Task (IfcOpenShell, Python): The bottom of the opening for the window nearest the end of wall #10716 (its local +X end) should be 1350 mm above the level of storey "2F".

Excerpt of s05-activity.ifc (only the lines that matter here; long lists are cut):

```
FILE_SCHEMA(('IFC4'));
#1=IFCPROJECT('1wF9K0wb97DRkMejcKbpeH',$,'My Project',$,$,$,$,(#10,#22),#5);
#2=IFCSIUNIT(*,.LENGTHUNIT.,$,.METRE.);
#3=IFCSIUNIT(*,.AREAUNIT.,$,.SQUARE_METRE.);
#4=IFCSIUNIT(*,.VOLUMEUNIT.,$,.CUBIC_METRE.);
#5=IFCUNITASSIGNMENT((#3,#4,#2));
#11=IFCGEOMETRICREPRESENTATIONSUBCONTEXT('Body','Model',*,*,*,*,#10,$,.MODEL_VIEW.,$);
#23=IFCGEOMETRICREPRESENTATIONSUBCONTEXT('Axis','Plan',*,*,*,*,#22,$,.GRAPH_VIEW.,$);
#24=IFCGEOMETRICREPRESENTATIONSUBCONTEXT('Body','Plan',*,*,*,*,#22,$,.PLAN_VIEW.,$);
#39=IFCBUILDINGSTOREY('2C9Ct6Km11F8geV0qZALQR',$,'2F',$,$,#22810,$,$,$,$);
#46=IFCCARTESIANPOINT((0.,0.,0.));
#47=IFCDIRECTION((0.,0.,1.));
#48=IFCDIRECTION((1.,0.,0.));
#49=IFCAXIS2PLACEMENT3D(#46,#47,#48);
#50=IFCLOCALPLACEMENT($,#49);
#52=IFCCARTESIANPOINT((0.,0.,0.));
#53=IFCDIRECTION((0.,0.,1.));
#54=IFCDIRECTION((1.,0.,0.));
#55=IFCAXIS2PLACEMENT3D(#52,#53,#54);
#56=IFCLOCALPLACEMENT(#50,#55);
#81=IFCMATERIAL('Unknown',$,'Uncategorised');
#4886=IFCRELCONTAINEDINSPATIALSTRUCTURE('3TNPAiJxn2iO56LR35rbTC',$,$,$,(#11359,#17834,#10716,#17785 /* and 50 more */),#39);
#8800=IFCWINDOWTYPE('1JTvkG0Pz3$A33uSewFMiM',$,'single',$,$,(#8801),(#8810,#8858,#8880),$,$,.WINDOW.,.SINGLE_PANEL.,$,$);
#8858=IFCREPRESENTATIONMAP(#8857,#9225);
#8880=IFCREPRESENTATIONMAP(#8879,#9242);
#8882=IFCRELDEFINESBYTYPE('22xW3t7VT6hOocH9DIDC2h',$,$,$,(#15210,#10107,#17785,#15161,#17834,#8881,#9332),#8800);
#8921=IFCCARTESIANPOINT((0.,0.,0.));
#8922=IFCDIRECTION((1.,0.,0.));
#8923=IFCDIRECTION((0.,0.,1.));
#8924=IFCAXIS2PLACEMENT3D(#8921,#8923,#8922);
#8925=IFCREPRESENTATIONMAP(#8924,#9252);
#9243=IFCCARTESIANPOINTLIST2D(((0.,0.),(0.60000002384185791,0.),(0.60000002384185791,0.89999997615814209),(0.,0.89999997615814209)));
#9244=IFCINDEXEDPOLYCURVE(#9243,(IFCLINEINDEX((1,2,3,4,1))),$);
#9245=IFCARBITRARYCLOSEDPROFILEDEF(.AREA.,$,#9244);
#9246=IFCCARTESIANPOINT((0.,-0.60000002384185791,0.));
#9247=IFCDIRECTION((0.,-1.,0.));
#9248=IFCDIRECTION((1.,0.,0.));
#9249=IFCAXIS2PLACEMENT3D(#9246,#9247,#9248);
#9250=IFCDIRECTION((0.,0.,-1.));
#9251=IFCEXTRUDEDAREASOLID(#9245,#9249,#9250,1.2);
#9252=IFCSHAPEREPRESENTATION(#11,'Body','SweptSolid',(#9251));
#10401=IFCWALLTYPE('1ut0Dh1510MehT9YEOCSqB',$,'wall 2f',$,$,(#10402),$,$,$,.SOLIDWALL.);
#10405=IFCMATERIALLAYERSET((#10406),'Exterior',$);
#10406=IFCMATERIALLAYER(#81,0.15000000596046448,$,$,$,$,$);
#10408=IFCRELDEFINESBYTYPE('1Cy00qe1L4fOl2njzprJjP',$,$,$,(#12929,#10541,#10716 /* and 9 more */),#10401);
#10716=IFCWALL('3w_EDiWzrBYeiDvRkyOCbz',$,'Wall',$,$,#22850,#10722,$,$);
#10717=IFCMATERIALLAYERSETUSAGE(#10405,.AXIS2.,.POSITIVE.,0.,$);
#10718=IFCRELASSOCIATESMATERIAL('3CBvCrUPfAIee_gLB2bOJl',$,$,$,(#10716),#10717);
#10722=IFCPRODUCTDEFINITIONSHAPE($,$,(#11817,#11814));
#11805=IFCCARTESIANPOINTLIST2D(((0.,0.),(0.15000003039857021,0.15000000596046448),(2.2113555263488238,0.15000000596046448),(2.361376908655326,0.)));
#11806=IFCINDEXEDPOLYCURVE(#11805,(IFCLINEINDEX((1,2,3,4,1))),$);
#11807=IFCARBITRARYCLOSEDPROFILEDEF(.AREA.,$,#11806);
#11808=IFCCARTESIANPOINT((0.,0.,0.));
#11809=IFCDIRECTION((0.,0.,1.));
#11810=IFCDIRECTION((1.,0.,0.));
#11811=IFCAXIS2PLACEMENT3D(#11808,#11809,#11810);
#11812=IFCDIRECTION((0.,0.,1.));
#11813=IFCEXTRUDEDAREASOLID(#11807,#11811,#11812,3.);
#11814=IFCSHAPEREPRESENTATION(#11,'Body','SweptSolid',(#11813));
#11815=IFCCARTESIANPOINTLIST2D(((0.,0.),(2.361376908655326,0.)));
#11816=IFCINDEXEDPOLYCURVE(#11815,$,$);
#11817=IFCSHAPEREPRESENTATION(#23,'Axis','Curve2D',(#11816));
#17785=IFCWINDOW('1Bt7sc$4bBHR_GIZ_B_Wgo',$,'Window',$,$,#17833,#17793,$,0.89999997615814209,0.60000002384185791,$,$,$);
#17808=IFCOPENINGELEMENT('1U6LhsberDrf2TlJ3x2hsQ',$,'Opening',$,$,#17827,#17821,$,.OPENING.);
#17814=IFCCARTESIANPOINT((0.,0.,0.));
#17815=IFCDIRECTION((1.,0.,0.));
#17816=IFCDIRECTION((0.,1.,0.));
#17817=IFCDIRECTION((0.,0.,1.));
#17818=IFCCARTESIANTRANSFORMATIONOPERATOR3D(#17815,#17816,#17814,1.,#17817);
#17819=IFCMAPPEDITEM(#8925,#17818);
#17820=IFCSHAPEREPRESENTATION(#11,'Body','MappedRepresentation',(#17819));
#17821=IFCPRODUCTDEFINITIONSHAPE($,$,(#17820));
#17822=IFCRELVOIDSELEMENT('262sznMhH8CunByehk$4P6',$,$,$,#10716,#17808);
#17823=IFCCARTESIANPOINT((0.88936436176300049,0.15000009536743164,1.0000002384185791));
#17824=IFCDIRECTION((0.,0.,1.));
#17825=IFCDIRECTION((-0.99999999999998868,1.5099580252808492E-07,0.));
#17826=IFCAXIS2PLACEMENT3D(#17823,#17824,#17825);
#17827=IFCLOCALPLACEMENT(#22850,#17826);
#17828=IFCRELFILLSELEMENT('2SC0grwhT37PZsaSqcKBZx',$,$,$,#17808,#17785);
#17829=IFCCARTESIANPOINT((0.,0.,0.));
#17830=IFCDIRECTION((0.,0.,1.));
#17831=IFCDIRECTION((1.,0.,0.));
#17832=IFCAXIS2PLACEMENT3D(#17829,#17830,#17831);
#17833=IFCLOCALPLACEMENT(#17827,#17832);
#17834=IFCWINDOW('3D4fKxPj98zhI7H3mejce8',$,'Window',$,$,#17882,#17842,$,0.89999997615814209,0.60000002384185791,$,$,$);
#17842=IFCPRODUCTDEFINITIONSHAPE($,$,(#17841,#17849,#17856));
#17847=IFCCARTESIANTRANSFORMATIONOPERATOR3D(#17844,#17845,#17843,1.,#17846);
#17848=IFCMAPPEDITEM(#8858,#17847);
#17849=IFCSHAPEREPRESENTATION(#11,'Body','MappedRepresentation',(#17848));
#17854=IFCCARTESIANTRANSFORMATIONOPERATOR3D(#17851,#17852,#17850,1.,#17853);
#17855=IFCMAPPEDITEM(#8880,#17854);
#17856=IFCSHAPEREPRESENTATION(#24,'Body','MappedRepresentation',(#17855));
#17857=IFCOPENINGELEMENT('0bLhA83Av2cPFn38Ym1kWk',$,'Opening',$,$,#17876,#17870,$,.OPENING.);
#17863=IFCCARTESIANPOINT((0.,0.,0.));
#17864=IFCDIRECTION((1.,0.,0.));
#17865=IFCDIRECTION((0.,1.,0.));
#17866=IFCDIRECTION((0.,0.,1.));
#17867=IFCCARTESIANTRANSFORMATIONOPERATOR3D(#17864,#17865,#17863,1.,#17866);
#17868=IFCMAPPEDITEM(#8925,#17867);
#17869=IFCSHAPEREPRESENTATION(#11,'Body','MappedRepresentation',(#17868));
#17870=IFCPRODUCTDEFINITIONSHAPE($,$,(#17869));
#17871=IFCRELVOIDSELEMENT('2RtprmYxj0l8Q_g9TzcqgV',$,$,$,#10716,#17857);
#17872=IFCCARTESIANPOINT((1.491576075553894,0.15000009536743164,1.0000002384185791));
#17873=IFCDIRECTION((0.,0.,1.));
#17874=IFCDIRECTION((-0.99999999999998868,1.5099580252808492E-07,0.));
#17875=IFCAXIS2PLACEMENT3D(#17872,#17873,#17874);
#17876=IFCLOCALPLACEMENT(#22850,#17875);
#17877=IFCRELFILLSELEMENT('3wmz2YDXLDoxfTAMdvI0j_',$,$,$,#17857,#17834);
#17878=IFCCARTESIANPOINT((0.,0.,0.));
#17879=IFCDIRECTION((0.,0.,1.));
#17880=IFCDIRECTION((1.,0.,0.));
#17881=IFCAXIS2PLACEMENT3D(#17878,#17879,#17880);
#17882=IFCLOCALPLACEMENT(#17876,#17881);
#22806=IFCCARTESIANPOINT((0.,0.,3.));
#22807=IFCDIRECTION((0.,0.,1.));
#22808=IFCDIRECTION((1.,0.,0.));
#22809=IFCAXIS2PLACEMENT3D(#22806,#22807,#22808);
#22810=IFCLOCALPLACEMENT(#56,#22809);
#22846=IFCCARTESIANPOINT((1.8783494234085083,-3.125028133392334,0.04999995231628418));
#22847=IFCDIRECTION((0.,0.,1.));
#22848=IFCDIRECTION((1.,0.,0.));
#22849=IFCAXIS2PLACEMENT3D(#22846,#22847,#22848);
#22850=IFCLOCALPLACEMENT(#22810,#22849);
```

```python
import numpy as np
import ifcopenshell
import ifcopenshell.api.geometry
import ifcopenshell.geom
import ifcopenshell.util.element
import ifcopenshell.util.placement
import ifcopenshell.util.shape
import ifcopenshell.util.unit

model = ifcopenshell.open("s05-activity.ifc")
unit_scale = ifcopenshell.util.unit.calculate_unit_scale(model)

window = model.by_guid("3D4fKxPj98zhI7H3mejce8")
opening = window.FillsVoids[0].RelatingOpeningElement
storey = ifcopenshell.util.element.get_container(window, ifc_class="IfcBuildingStorey")
level = ifcopenshell.util.placement.get_local_placement(storey.ObjectPlacement)[2, 3]

# The opening's origin need not be at the sill, so measure its lowest point.
shape = ifcopenshell.geom.create_shape(ifcopenshell.geom.settings(), opening)
bottom = ifcopenshell.util.shape.get_shape_bottom_elevation(shape, shape.geometry) / unit_scale
dz = level + 1.35 / unit_scale - bottom

shift = np.array([0.0, 0.0, dz])
# The window is placed relative to its opening, so it follows when the opening moves.
matrix = ifcopenshell.util.placement.get_local_placement(opening.ObjectPlacement)
matrix[:3, 3] += shift
ifcopenshell.api.geometry.edit_object_placement(
    model, product=opening, matrix=matrix, is_si=False, should_transform_children=True
)

print(f"moved by {dz * unit_scale:+.3f} m")

model.write("s05-activity-out.ifc")
```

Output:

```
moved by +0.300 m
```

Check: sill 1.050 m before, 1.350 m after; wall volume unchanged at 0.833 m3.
